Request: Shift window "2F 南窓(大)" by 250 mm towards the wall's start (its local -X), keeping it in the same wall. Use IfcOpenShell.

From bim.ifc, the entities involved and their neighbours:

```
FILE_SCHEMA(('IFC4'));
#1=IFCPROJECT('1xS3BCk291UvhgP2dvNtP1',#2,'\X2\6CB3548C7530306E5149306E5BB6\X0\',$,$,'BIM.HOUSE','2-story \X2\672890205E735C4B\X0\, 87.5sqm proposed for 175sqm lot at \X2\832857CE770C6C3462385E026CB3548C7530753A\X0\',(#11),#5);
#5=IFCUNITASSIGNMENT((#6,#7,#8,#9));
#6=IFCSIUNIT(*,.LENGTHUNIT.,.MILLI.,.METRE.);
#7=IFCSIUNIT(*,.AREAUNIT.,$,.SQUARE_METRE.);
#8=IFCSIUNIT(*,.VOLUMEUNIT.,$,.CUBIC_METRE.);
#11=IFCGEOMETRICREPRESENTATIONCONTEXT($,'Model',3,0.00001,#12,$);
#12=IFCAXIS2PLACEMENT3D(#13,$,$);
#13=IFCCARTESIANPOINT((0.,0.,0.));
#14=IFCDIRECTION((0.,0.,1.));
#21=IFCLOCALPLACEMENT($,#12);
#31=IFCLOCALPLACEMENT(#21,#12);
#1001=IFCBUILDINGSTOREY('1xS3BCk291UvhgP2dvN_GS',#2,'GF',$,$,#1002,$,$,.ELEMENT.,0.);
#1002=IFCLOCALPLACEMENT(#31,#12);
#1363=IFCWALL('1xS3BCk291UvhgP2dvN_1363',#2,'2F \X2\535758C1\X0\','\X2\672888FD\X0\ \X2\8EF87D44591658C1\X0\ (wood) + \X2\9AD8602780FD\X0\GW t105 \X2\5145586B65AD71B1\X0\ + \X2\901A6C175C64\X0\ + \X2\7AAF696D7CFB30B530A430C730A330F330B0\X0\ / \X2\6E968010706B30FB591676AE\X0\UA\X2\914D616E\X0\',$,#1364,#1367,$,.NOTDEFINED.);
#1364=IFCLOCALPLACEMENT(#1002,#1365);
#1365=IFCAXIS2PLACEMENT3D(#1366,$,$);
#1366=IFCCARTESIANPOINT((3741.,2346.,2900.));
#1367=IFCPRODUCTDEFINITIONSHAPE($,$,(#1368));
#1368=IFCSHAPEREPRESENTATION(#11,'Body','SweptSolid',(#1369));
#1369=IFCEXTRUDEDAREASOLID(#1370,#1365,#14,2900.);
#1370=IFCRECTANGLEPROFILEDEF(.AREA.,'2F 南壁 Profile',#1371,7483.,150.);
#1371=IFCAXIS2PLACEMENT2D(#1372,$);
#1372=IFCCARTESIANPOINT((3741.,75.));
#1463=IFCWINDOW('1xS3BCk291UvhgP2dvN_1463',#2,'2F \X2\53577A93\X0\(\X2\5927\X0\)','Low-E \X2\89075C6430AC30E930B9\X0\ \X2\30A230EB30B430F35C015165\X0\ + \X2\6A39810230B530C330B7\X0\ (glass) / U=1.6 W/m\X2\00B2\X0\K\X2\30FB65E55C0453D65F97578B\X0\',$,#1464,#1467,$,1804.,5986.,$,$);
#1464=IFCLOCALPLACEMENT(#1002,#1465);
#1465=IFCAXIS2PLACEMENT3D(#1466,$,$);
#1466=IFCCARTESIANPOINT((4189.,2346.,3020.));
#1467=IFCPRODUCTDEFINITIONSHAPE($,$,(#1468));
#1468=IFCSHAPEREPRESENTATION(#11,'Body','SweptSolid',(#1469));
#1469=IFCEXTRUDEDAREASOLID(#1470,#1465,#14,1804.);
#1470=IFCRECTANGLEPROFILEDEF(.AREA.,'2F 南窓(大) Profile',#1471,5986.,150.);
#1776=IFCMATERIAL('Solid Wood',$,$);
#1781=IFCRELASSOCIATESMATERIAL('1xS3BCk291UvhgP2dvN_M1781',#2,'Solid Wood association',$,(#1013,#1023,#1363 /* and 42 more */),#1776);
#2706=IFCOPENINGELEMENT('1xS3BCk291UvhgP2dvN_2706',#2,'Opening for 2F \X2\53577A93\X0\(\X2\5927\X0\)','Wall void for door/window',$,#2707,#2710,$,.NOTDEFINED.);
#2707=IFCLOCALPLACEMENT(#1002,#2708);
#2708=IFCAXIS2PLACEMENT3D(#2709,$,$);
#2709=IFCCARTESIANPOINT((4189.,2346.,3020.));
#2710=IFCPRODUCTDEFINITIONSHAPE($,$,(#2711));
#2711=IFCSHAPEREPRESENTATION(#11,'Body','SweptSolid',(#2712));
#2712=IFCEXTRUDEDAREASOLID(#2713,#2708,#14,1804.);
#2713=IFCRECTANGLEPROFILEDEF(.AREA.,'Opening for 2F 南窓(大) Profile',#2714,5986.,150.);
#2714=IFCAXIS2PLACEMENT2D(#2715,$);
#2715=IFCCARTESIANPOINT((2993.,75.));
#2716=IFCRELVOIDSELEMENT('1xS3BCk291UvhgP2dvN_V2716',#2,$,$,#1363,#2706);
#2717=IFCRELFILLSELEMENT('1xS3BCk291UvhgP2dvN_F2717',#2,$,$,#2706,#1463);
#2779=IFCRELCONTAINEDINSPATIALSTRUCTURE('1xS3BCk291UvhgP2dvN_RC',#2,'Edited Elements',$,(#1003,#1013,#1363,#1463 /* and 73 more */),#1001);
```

```python
import ifcopenshell
import ifcopenshell.api.geometry
import ifcopenshell.util.placement
import ifcopenshell.util.unit

model = ifcopenshell.open("bim.ifc")
unit_scale = ifcopenshell.util.unit.calculate_unit_scale(model)

window = model.by_guid("1xS3BCk291UvhgP2dvN_1463")
opening = window.FillsVoids[0].RelatingOpeningElement
wall = opening.VoidsElements[0].RelatingBuildingElement

wall_matrix = ifcopenshell.util.placement.get_local_placement(wall.ObjectPlacement)
shift = wall_matrix[:3, 0] * -0.25 / unit_scale
before = ifcopenshell.util.placement.get_local_placement(window.ObjectPlacement)[:3, 3].copy()

# The window is not placed relative to its opening, so move both.
for product in (opening, window):
    matrix = ifcopenshell.util.placement.get_local_placement(product.ObjectPlacement)
    matrix[:3, 3] += shift
    ifcopenshell.api.geometry.edit_object_placement(model, product=product, matrix=matrix, is_si=False)

after = ifcopenshell.util.placement.get_local_placement(window.ObjectPlacement)[:3, 3]
print("window moved by", (after - before).round(3) + 0.0)

model.write("bim-out.ifc")
```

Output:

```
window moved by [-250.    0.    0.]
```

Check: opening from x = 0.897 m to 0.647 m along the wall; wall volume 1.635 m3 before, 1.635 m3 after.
